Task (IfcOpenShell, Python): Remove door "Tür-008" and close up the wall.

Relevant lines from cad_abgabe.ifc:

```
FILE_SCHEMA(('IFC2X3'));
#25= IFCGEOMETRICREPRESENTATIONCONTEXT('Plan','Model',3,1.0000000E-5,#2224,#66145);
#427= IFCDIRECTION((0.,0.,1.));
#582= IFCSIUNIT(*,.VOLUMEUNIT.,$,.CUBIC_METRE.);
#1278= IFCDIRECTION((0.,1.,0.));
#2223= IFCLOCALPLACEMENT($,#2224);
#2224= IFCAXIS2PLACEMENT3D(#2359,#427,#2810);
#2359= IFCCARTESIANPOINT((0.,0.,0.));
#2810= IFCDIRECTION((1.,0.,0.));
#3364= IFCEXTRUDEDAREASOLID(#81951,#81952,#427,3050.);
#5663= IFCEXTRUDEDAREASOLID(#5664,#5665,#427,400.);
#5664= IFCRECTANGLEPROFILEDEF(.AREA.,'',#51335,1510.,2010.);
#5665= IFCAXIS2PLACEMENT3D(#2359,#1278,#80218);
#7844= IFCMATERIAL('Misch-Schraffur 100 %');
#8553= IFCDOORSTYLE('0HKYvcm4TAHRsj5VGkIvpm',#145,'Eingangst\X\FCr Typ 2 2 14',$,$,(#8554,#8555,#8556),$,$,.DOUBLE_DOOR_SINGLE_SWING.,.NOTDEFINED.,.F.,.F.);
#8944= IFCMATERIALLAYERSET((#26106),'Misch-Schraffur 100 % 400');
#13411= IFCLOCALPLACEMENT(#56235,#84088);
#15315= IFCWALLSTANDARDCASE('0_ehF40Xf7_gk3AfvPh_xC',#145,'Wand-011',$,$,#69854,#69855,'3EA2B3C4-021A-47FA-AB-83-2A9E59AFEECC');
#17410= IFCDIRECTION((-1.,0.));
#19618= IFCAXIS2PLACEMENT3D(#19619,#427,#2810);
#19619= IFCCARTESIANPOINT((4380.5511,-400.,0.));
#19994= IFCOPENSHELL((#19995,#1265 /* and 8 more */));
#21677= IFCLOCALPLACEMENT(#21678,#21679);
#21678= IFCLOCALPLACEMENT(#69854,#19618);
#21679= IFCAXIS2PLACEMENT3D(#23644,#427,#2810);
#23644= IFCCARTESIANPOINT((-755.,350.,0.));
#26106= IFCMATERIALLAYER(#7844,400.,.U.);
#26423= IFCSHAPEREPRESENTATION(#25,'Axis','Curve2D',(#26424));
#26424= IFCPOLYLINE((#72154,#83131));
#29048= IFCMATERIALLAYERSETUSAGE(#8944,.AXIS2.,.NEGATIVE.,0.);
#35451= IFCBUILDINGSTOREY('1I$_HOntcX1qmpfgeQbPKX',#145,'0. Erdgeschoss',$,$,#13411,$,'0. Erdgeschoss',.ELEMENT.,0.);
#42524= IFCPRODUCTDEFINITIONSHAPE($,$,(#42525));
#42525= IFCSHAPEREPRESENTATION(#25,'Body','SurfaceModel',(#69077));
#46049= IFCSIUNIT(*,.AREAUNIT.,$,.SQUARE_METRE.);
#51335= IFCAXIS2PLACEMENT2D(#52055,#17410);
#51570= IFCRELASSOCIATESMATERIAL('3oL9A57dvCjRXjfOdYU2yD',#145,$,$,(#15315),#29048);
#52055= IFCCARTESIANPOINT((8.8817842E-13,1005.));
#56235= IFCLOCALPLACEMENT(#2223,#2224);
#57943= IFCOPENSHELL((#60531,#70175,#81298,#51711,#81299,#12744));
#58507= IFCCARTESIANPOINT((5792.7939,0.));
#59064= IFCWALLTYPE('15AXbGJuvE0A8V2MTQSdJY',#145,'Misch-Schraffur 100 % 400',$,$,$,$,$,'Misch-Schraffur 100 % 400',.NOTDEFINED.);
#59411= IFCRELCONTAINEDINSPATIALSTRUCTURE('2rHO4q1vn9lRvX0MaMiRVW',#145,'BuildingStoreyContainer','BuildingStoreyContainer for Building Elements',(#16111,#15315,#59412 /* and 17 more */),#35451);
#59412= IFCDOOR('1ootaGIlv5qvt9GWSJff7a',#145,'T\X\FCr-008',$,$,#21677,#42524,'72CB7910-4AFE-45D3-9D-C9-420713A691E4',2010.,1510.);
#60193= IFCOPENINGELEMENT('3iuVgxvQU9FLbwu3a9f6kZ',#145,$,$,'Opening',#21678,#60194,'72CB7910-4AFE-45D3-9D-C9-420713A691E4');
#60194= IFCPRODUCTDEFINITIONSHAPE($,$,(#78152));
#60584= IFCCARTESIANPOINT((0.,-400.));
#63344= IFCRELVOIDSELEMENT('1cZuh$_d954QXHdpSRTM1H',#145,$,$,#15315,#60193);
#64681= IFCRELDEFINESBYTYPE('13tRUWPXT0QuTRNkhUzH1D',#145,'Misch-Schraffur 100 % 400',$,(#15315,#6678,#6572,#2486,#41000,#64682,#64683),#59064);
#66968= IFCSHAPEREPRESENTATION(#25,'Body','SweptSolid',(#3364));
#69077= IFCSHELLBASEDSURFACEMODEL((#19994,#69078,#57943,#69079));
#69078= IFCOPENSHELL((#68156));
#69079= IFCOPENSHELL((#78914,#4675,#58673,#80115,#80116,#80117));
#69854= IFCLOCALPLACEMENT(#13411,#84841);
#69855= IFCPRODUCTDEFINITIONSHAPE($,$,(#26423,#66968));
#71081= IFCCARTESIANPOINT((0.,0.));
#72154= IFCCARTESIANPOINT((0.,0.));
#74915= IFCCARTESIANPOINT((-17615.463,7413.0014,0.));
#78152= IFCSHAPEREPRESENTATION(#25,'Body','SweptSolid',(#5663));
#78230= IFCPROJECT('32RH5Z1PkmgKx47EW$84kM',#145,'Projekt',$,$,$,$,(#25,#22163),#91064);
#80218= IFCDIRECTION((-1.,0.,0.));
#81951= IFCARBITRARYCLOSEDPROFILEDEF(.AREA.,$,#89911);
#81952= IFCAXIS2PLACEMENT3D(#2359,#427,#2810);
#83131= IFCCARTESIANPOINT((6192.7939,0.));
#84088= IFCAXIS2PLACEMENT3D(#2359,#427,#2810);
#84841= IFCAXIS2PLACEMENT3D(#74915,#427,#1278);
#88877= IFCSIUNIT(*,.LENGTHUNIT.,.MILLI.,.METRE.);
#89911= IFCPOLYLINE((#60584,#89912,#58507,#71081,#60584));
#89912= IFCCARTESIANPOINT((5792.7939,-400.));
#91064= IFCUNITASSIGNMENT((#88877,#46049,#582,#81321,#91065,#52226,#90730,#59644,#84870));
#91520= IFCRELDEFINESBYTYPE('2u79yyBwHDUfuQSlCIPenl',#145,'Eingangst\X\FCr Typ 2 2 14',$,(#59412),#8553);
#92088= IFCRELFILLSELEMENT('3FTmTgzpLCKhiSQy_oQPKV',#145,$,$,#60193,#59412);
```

```python
import ifcopenshell
import ifcopenshell.api.feature
import ifcopenshell.api.root
import ifcopenshell.geom
import ifcopenshell.util.shape

model = ifcopenshell.open("cad_abgabe.ifc")
settings = ifcopenshell.geom.settings()


def volume(element):
    """Net volume in cubic metres, openings subtracted."""
    shape = ifcopenshell.geom.create_shape(settings, element)
    return ifcopenshell.util.shape.get_volume(shape.geometry)


door = model.by_id(59412)
opening = door.FillsVoids[0].RelatingOpeningElement
wall = opening.VoidsElements[0].RelatingBuildingElement
before = volume(wall)

ifcopenshell.api.root.remove_product(model, product=door)
ifcopenshell.api.feature.remove_feature(model, feature=opening)

after = volume(wall)

print(f"wall volume {before:.3f} -> {after:.3f} m3")

model.write("cad_abgabe_updated.ifc")
```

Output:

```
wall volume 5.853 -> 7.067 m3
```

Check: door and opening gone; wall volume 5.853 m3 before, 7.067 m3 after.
